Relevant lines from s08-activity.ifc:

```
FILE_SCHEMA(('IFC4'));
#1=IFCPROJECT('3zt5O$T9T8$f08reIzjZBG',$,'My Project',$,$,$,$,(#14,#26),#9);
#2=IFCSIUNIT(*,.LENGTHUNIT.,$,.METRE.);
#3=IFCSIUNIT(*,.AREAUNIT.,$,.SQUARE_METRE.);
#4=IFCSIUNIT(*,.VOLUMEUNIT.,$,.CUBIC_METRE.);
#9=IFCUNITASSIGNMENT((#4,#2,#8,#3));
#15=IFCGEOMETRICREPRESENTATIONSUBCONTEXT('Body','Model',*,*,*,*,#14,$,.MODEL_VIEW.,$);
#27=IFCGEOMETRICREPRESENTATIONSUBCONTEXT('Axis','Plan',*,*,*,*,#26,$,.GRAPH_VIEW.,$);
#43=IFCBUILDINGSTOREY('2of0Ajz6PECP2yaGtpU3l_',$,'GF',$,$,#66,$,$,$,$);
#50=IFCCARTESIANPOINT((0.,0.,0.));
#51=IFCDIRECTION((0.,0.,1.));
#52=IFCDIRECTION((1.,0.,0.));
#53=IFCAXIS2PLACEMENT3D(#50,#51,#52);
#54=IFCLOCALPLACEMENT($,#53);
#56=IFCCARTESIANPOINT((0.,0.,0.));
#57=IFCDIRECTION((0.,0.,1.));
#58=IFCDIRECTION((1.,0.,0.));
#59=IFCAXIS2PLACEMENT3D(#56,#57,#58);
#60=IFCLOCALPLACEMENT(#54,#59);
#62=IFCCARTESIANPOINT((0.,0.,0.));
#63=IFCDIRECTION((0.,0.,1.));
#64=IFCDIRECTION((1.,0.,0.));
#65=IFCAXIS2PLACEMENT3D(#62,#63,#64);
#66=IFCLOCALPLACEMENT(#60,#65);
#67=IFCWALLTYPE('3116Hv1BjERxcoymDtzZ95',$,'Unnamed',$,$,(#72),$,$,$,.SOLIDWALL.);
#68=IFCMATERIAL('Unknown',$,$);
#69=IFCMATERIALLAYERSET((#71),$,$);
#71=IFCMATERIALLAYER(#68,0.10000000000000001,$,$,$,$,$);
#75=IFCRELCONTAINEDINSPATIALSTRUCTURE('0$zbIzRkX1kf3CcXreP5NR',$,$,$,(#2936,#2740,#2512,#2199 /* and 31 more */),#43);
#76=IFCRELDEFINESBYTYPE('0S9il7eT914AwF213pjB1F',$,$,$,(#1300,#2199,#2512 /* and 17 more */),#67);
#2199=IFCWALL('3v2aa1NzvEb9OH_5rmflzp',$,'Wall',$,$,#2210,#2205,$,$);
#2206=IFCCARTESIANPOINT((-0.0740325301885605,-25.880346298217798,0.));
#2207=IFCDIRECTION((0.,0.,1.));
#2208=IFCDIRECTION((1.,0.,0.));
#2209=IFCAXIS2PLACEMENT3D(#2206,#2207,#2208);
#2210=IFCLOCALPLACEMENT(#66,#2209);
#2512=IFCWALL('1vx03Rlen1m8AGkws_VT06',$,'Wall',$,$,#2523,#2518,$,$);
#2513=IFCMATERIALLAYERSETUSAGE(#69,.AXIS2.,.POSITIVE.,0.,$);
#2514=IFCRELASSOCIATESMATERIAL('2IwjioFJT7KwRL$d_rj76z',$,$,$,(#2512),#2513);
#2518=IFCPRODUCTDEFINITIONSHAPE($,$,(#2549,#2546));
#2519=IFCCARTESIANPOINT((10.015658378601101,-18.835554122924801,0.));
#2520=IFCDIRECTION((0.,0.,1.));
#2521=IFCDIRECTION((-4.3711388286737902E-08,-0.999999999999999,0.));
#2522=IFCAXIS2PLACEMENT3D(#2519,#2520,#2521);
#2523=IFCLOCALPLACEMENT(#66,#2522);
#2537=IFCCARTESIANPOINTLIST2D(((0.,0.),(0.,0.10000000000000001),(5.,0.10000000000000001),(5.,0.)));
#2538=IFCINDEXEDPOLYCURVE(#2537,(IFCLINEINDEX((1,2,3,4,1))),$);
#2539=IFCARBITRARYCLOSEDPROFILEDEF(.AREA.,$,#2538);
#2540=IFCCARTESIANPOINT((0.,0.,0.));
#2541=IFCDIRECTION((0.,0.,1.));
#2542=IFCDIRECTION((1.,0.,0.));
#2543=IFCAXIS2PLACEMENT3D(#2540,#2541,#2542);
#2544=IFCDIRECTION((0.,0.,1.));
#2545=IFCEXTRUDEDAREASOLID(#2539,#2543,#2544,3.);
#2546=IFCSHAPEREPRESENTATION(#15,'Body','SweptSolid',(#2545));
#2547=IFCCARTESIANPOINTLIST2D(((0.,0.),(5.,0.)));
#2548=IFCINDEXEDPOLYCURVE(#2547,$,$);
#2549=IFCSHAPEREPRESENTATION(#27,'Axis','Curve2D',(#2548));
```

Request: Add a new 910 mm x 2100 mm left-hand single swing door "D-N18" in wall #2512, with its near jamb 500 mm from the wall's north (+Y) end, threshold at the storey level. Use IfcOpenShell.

```python
import numpy as np
import ifcopenshell
import ifcopenshell.api.feature
import ifcopenshell.api.geometry
import ifcopenshell.api.root
import ifcopenshell.api.spatial
import ifcopenshell.geom
import ifcopenshell.util.element
import ifcopenshell.util.placement
import ifcopenshell.util.representation
import ifcopenshell.util.shape
import ifcopenshell.util.unit

model = ifcopenshell.open("s08-activity.ifc")
unit_scale = ifcopenshell.util.unit.calculate_unit_scale(model)
settings = ifcopenshell.geom.settings()


def volume(element):
    """Net volume in cubic metres, openings subtracted."""
    shape = ifcopenshell.geom.create_shape(settings, element)
    return ifcopenshell.util.shape.get_volume(shape.geometry)


wall = model.by_id(2512)
storey = ifcopenshell.util.element.get_container(wall, ifc_class="IfcBuildingStorey")
context = ifcopenshell.util.representation.get_context(model, "Model", "Body", "MODEL_VIEW")
before = volume(wall)

width, height, from_end, sill = 0.91, 2.1, 0.5, 0.0  # metres

# The wall runs along its own X axis, and the end named is its -X end.
wall_shape = ifcopenshell.geom.create_shape(settings, wall)
x, y, z = ifcopenshell.util.shape.get_vertices(wall_shape.geometry).T
start = x.min() + from_end
face, thickness = float(y.min()), float(y.max() - y.min())
wall_matrix = ifcopenshell.util.placement.get_local_placement(wall.ObjectPlacement)
level = ifcopenshell.util.placement.get_local_placement(storey.ObjectPlacement)[2, 3]


def in_wall(x, y):
    """Placement at x, y metres in the wall's axes, at sill height."""
    matrix = wall_matrix.copy()
    matrix[:, 3] = wall_matrix @ np.array([x / unit_scale, y / unit_scale, 0.0, 1.0])
    matrix[2, 3] = level + sill / unit_scale
    return matrix


# Opening: a box that overshoots both wall faces by 50 mm.
opening = ifcopenshell.api.root.create_entity(model, ifc_class="IfcOpeningElement", predefined_type="OPENING")
box = ifcopenshell.api.geometry.add_wall_representation(
    model, context=context, length=width, height=height, thickness=thickness + 0.1
)
ifcopenshell.api.geometry.assign_representation(model, product=opening, representation=box)
ifcopenshell.api.geometry.edit_object_placement(model, product=opening, matrix=in_wall(start, face - 0.05), is_si=False)
ifcopenshell.api.feature.add_feature(model, feature=opening, element=wall)

door = ifcopenshell.api.root.create_entity(model, ifc_class="IfcDoor", name="D-N18", predefined_type="DOOR")
door.OverallWidth, door.OverallHeight = width / unit_scale, height / unit_scale
door.OperationType = "SINGLE_SWING_LEFT"
body = ifcopenshell.api.geometry.add_door_representation(
    model,
    context=context,
    overall_width=door.OverallWidth,
    overall_height=door.OverallHeight,
    operation_type="SINGLE_SWING_LEFT",
    lining_properties={"LiningDepth": thickness / unit_scale, "ThresholdDepth": thickness / unit_scale},
)
ifcopenshell.api.geometry.assign_representation(model, product=door, representation=body)
ifcopenshell.api.spatial.assign_container(model, products=[door], relating_structure=storey)
ifcopenshell.api.feature.add_filling(model, opening=opening, element=door)

# The lining spans the wall, so the door starts at the wall face.
ifcopenshell.api.geometry.edit_object_placement(model, product=door, matrix=in_wall(start, face), is_si=False)

after = volume(wall)

print(f"wall volume {before:.3f} -> {after:.3f} m3")

model.write("s08-activity_rev.ifc")
```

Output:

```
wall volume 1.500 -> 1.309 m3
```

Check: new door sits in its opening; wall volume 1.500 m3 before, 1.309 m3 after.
